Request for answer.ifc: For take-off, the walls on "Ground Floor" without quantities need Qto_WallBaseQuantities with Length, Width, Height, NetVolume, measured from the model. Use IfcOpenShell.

First a look at what the model holds.

```python
import ifcopenshell
import ifcopenshell.util.element
import ifcopenshell.util.unit

model = ifcopenshell.open("answer.ifc")
print(model.schema)
for unit_type in ("LENGTHUNIT", "AREAUNIT", "VOLUMEUNIT"):
    print(unit_type, ifcopenshell.util.unit.calculate_unit_scale(model, unit_type))
storey = next(s for s in model.by_type("IfcBuildingStorey") if s.Name == "Ground Floor")
walls = [e for e in ifcopenshell.util.element.get_decomposition(storey) if e.is_a("IfcWall")]
for e in sorted(walls, key=lambda e: e.id()):
    print(e.id(), e.is_a(), e.Name, list(ifcopenshell.util.element.get_psets(e, qtos_only=True)), sep=" | ")
```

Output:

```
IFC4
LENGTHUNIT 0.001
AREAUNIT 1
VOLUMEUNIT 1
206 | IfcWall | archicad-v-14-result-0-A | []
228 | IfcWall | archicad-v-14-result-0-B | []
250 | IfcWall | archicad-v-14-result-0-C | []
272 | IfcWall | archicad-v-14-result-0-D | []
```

```python
import ifcopenshell
import ifcopenshell.api.pset
import ifcopenshell.geom
import ifcopenshell.util.element
import ifcopenshell.util.shape
import ifcopenshell.util.unit

model = ifcopenshell.open("answer.ifc")
unit_scale = ifcopenshell.util.unit.calculate_unit_scale(model)
volume_scale = ifcopenshell.util.unit.calculate_unit_scale(model, "VOLUMEUNIT")
settings = ifcopenshell.geom.settings()

storey = next(s for s in model.by_type("IfcBuildingStorey") if s.Name == "Ground Floor")
walls = [e for e in ifcopenshell.util.element.get_decomposition(storey) if e.is_a("IfcWall")]

for e in sorted(walls, key=lambda e: e.id()):
    if ifcopenshell.util.element.get_psets(e, qtos_only=True, should_inherit=False):
        continue
    # Geometry comes back in metres, in the element's own axes.
    shape = ifcopenshell.geom.create_shape(settings, e)
    values = {
        "Length": ifcopenshell.util.shape.get_x(shape.geometry) / unit_scale,
        "Width": ifcopenshell.util.shape.get_y(shape.geometry) / unit_scale,
        "Height": ifcopenshell.util.shape.get_z(shape.geometry) / unit_scale,
        "NetVolume": ifcopenshell.util.shape.get_volume(shape.geometry) / volume_scale,
    }
    qto = ifcopenshell.api.pset.add_qto(model, product=e, name="Qto_WallBaseQuantities")
    ifcopenshell.api.pset.edit_qto(model, qto=qto, properties=values)
    print(e.id(), {k: round(v, 3) for k, v in values.items()})

model.write("answer_rev.ifc")
```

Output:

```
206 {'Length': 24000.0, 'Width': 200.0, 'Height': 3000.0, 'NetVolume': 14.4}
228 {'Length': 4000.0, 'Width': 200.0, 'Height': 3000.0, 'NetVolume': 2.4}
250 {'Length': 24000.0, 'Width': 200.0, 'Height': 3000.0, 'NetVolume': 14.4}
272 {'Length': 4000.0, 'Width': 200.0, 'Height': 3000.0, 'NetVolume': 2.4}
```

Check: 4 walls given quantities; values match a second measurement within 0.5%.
